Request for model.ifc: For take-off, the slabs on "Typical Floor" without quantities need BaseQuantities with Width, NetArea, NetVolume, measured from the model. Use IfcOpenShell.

First a look at what the model holds.

```python
import ifcopenshell
import ifcopenshell.util.element
import ifcopenshell.util.unit

model = ifcopenshell.open("model.ifc")
print(model.schema)
for unit_type in ("LENGTHUNIT", "AREAUNIT", "VOLUMEUNIT"):
    print(unit_type, ifcopenshell.util.unit.calculate_unit_scale(model, unit_type))
storey = next(s for s in model.by_type("IfcBuildingStorey") if s.Name == "Typical Floor")
slabs = [e for e in ifcopenshell.util.element.get_decomposition(storey) if e.is_a("IfcSlab")]
for e in sorted(slabs, key=lambda e: e.id()):
    print(e.id(), e.is_a(), e.Name, list(ifcopenshell.util.element.get_psets(e, qtos_only=True)), sep=" | ")
```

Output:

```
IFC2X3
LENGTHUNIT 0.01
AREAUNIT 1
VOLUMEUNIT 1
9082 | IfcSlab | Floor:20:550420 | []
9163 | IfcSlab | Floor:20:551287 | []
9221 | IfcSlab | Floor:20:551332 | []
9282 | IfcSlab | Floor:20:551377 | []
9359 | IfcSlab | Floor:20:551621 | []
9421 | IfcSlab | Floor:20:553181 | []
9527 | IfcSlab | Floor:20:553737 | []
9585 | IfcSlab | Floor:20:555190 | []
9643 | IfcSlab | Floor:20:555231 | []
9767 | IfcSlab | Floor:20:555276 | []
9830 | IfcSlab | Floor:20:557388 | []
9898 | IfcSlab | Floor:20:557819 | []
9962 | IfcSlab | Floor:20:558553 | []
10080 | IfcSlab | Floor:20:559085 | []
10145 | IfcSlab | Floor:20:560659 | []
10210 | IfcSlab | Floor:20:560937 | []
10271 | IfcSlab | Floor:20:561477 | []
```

```python
import ifcopenshell
import ifcopenshell.api.pset
import ifcopenshell.geom
import ifcopenshell.util.element
import ifcopenshell.util.shape
import ifcopenshell.util.unit

model = ifcopenshell.open("model.ifc")
unit_scale = ifcopenshell.util.unit.calculate_unit_scale(model)
area_scale = ifcopenshell.util.unit.calculate_unit_scale(model, "AREAUNIT")
volume_scale = ifcopenshell.util.unit.calculate_unit_scale(model, "VOLUMEUNIT")
settings = ifcopenshell.geom.settings()

storey = next(s for s in model.by_type("IfcBuildingStorey") if s.Name == "Typical Floor")
slabs = [e for e in ifcopenshell.util.element.get_decomposition(storey) if e.is_a("IfcSlab")]

for e in sorted(slabs, key=lambda e: e.id()):
    if ifcopenshell.util.element.get_psets(e, qtos_only=True, should_inherit=False):
        continue
    # Geometry comes back in metres, in the element's own axes.
    shape = ifcopenshell.geom.create_shape(settings, e)
    values = {
        "Width": ifcopenshell.util.shape.get_z(shape.geometry) / unit_scale,
        "NetArea": ifcopenshell.util.shape.get_footprint_area(shape.geometry) / area_scale,
        "NetVolume": ifcopenshell.util.shape.get_volume(shape.geometry) / volume_scale,
    }
    qto = ifcopenshell.api.pset.add_qto(model, product=e, name="BaseQuantities")
    ifcopenshell.api.pset.edit_qto(model, qto=qto, properties=values)
    print(e.id(), {k: round(v, 3) for k, v in values.items()})

model.write("model-out.ifc")
```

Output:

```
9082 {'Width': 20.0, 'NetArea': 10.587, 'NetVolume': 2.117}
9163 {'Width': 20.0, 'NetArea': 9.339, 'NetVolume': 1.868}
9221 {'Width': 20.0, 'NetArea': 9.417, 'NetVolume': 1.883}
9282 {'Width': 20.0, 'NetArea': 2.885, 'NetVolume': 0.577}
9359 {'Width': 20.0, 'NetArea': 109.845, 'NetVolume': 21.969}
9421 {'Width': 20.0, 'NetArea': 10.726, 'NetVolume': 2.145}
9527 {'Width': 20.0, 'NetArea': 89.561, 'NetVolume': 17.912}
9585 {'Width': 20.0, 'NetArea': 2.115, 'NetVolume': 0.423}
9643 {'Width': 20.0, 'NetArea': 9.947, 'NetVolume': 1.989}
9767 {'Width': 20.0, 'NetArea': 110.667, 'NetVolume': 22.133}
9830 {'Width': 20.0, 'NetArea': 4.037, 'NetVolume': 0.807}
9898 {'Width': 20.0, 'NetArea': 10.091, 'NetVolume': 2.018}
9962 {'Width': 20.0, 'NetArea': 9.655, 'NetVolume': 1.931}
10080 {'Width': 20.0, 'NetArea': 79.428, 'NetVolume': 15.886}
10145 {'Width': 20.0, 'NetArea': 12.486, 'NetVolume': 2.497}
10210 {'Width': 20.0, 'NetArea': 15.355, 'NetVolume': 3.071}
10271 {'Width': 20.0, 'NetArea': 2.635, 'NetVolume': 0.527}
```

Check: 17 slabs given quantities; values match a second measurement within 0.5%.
